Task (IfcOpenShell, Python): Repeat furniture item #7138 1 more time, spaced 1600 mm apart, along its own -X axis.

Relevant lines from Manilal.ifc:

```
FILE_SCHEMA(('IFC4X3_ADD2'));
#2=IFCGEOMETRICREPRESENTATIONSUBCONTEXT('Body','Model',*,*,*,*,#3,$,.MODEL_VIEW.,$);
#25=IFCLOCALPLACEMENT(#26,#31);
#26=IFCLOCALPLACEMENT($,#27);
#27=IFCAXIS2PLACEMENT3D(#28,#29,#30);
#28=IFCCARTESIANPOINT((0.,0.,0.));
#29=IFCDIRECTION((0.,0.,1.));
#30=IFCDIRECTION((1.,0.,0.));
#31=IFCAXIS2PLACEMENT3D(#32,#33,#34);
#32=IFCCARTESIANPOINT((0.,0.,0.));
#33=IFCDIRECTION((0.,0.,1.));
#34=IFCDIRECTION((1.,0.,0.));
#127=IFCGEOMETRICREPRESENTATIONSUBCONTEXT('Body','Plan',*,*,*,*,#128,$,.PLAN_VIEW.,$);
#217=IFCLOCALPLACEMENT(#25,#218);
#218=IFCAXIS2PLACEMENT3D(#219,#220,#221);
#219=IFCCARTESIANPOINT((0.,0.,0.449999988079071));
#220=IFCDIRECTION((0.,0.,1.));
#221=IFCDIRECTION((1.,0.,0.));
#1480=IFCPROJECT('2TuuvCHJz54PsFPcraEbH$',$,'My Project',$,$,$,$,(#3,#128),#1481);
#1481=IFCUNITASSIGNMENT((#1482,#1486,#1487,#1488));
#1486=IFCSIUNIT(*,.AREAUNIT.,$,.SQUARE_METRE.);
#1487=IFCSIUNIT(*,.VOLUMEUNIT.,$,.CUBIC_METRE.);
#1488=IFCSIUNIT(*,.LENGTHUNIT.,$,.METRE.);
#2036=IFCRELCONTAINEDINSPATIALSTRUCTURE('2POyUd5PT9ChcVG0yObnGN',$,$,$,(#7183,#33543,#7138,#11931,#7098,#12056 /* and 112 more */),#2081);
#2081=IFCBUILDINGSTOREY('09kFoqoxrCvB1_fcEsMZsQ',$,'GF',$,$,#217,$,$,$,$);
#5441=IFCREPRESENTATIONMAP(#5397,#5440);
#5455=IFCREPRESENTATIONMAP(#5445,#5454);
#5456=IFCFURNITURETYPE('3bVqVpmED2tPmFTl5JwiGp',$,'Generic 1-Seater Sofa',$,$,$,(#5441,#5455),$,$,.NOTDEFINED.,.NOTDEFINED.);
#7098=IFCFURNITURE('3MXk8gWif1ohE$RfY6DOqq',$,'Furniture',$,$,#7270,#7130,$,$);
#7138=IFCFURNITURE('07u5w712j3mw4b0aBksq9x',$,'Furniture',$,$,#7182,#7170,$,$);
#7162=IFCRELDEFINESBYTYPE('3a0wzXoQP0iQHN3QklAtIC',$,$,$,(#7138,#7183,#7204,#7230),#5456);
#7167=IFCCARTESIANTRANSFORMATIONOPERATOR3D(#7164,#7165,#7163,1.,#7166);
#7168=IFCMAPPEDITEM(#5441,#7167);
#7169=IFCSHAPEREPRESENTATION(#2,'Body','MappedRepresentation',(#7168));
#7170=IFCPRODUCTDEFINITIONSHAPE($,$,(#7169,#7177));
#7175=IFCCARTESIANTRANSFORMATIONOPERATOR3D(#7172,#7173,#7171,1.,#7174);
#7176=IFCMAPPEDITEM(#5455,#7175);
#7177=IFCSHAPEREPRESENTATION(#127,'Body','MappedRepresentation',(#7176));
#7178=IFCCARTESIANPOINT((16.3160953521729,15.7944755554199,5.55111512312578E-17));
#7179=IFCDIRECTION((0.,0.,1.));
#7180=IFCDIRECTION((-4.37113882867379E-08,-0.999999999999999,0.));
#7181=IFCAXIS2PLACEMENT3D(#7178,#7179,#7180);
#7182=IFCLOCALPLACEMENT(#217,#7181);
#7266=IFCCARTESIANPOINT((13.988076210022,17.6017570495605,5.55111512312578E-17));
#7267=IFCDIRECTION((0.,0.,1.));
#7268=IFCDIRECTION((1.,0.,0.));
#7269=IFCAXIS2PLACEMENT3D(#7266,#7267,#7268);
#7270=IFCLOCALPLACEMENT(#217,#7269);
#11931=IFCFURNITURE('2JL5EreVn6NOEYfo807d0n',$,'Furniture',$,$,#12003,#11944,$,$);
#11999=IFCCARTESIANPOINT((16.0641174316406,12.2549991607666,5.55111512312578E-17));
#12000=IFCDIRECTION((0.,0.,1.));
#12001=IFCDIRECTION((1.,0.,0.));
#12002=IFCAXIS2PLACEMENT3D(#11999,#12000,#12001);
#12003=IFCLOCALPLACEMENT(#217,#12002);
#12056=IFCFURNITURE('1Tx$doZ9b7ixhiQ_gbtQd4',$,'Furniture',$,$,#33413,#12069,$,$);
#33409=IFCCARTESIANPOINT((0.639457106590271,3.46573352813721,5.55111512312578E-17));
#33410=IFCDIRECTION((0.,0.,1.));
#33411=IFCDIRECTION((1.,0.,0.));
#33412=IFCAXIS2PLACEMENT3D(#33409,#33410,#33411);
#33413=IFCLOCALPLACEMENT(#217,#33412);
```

```python
import ifcopenshell
import ifcopenshell.api.geometry
import ifcopenshell.api.root
import ifcopenshell.util.element
import ifcopenshell.util.placement
import ifcopenshell.util.unit

model = ifcopenshell.open("Manilal.ifc")
unit_scale = ifcopenshell.util.unit.calculate_unit_scale(model)

source = model.by_guid("07u5w712j3mw4b0aBksq9x")
base = ifcopenshell.util.placement.get_local_placement(source.ObjectPlacement)
step = -base[:3, 0] * 1.6 / unit_scale

for i in range(1, 2):
    copy = ifcopenshell.api.root.copy_class(model, product=source)
    copy.Representation = ifcopenshell.util.element.copy_deep(
        model, source.Representation, exclude=["IfcGeometricRepresentationContext", "IfcRepresentationMap"]
    )
    matrix = base.copy()
    matrix[:3, 3] += i * step
    print("added at", matrix[:3, 3].round(3) + 0.0)
    ifcopenshell.api.geometry.edit_object_placement(model, product=copy, matrix=matrix, is_si=False)

model.write("Manilal_v2.ifc")
```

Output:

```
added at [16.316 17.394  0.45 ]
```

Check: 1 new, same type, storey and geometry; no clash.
